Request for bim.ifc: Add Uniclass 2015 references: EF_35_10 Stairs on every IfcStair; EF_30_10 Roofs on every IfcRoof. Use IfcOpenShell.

First a look at what the model holds.

```python
import ifcopenshell

model = ifcopenshell.open("bim.ifc")
print(model.schema)
print("classifications:", [c.Name for c in model.by_type("IfcClassification")])
for ifc_class in ("IfcDoor", "IfcRoof", "IfcStair", "IfcWall", "IfcWindow"):
    print(ifc_class, len(model.by_type(ifc_class)))
```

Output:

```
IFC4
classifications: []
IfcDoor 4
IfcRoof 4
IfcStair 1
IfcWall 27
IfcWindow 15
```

```python
import ifcopenshell
import ifcopenshell.api.classification

model = ifcopenshell.open("bim.ifc")

system = ifcopenshell.api.classification.add_classification(model, classification="Uniclass 2015")

codes = {
    "IfcStair": ("EF_35_10", "Stairs"),
    "IfcRoof": ("EF_30_10", "Roofs"),
}
for ifc_class, (code, name) in codes.items():
    products = model.by_type(ifc_class)
    ifcopenshell.api.classification.add_reference(
        model, products=products, classification=system, identification=code, name=name
    )
    print(code, len(products))

model.write("bim_v2.ifc")
```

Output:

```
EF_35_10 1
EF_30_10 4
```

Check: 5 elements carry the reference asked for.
